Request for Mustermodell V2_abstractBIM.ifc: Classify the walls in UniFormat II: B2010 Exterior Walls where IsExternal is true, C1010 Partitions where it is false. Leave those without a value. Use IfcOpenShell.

First a look at what the model holds.

```python
import ifcopenshell
import ifcopenshell.util.element

model = ifcopenshell.open("Mustermodell V2_abstractBIM.ifc")
print(model.schema)
print("classifications:", [c.Name for c in model.by_type("IfcClassification")])
values = [ifcopenshell.util.element.get_pset(e, "Pset_WallCommon", "IsExternal") for e in model.by_type("IfcWall")]
for value in (True, False, None):
    print("IsExternal", value, values.count(value))
```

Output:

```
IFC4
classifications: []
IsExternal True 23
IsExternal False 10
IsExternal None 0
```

```python
import ifcopenshell
import ifcopenshell.api.classification
import ifcopenshell.util.element

model = ifcopenshell.open("Mustermodell V2_abstractBIM.ifc")

system = ifcopenshell.api.classification.add_classification(model, classification="UniFormat II")

walls = model.by_type("IfcWall")
external = {e: ifcopenshell.util.element.get_pset(e, "Pset_WallCommon", "IsExternal") for e in walls}
for flag, code, name in ((True, "B2010", "Exterior Walls"), (False, "C1010", "Partitions")):
    products = [e for e in walls if external[e] is flag]
    ifcopenshell.api.classification.add_reference(
        model, products=products, classification=system, identification=code, name=name
    )
    print(code, len(products))

model.write("Mustermodell V2_abstractBIM-out.ifc")
```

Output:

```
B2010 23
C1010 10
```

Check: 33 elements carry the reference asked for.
